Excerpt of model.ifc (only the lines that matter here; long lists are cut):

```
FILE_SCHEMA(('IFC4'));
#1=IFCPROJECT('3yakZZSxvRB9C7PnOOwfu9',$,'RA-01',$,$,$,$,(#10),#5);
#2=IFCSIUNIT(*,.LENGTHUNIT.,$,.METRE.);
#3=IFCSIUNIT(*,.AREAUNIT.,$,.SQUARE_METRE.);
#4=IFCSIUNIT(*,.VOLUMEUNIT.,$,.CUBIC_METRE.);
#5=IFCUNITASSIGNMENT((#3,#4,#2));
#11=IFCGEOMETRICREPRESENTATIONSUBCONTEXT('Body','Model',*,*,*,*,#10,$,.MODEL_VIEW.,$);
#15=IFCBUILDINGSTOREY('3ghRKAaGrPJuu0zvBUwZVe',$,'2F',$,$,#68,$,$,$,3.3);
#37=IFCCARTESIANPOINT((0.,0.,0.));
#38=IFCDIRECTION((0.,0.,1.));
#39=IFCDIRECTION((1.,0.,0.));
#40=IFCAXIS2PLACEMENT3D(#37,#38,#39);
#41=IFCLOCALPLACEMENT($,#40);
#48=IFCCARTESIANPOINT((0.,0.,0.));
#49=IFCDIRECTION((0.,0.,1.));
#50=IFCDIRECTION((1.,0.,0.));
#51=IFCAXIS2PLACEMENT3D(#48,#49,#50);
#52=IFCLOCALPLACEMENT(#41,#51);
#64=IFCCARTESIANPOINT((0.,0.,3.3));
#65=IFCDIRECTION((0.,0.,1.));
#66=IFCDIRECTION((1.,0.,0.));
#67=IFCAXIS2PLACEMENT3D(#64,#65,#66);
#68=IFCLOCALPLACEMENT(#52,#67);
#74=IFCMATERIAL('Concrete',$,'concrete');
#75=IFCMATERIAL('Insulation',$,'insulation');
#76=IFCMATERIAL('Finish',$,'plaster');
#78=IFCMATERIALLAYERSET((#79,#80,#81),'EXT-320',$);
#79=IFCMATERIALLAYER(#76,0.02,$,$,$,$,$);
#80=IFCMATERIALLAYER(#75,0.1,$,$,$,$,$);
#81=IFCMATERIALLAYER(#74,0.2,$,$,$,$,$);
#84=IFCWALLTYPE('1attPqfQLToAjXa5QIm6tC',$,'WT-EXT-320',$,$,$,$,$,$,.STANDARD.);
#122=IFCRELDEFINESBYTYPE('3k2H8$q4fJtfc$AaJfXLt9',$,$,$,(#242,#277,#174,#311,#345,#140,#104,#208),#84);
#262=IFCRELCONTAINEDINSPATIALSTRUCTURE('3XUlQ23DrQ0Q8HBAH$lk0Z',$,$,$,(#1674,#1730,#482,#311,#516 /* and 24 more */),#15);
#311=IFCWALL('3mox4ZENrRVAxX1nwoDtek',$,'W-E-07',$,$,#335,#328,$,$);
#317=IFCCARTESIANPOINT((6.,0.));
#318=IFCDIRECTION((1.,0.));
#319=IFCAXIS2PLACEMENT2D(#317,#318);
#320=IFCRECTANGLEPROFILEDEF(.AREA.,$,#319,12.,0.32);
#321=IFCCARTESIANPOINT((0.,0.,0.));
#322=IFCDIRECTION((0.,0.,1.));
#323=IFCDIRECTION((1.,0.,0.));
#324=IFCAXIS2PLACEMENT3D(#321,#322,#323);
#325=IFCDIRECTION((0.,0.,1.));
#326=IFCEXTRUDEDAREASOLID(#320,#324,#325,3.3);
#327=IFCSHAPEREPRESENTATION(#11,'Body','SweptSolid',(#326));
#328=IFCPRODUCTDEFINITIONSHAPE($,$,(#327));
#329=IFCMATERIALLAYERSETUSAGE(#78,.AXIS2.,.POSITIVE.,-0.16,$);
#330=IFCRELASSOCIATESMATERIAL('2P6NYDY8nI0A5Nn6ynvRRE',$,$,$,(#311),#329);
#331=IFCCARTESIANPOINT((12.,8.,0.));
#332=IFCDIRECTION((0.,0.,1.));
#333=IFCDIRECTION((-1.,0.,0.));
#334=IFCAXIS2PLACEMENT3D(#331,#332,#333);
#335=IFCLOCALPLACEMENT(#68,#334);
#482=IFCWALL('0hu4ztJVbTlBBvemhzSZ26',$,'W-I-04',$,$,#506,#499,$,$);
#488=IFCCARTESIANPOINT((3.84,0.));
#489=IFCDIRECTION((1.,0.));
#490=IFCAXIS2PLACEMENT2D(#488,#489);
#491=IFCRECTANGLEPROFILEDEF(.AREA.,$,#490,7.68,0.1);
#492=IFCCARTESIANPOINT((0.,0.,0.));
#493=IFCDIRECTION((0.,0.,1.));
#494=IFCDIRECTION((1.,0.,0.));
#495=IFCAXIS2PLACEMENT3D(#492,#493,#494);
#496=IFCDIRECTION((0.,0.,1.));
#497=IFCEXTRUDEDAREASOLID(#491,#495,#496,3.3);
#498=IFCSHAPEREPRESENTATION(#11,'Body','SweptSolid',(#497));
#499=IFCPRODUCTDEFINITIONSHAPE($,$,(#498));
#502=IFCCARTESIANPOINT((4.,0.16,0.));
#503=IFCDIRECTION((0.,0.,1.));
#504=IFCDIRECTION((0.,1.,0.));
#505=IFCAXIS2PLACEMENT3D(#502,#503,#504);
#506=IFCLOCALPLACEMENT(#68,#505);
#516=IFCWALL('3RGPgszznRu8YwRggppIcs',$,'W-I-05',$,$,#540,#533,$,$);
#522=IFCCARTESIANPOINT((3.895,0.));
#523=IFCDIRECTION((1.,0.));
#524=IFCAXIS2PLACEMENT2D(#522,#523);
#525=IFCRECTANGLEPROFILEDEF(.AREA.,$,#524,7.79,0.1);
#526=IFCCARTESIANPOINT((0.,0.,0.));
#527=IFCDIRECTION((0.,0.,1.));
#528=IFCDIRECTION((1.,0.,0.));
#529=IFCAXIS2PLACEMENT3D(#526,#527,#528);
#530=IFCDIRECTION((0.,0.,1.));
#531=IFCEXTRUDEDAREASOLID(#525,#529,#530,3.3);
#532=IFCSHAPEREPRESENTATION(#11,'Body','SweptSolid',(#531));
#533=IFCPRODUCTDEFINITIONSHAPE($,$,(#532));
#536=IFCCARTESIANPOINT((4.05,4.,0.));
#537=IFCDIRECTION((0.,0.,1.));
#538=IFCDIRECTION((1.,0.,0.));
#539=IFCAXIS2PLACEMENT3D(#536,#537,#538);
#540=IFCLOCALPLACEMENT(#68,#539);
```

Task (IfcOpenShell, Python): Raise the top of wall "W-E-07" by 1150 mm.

```python
import ifcopenshell
import ifcopenshell.geom
import ifcopenshell.util.representation
import ifcopenshell.util.shape
import ifcopenshell.util.unit

model = ifcopenshell.open("model.ifc")
unit_scale = ifcopenshell.util.unit.calculate_unit_scale(model)
settings = ifcopenshell.geom.settings()


def volume(element):
    """Net volume in cubic metres, openings subtracted."""
    shape = ifcopenshell.geom.create_shape(settings, element)
    return ifcopenshell.util.shape.get_volume(shape.geometry)


wall = model.by_id(311)
before = volume(wall)

body = ifcopenshell.util.representation.get_representation(wall, "Model", "Body")
solid = body.Items[0]
old_height = solid.Depth
solid.Depth += 1.15 / unit_scale
after = volume(wall)

print(f"height {old_height:g} -> {solid.Depth:g}, volume {before:.3f} -> {after:.3f} m3")

model.write("model_updated.ifc")
```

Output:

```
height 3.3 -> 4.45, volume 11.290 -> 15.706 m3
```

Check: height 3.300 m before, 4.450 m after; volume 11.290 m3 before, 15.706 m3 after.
